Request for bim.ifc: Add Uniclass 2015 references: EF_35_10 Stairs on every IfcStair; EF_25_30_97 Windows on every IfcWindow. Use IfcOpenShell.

First a look at what the model holds.

```python
import ifcopenshell

model = ifcopenshell.open("bim.ifc")
print(model.schema)
print("classifications:", [c.Name for c in model.by_type("IfcClassification")])
for ifc_class in ("IfcDoor", "IfcRoof", "IfcStair", "IfcWall", "IfcWindow"):
    print(ifc_class, len(model.by_type(ifc_class)))
```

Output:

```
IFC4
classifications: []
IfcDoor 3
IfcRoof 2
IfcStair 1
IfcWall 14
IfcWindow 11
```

```python
import ifcopenshell
import ifcopenshell.api.classification

model = ifcopenshell.open("bim.ifc")

system = ifcopenshell.api.classification.add_classification(model, classification="Uniclass 2015")

codes = {
    "IfcStair": ("EF_35_10", "Stairs"),
    "IfcWindow": ("EF_25_30_97", "Windows"),
}
for ifc_class, (code, name) in codes.items():
    products = model.by_type(ifc_class)
    ifcopenshell.api.classification.add_reference(
        model, products=products, classification=system, identification=code, name=name
    )
    print(code, len(products))

model.write("bim_edited.ifc")
```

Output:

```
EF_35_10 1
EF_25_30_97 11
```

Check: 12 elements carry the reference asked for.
